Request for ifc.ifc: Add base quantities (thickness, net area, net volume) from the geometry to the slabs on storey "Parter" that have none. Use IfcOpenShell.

First a look at what the model holds.

```python
import ifcopenshell
import ifcopenshell.util.element
import ifcopenshell.util.unit

model = ifcopenshell.open("ifc.ifc")
print(model.schema)
for unit_type in ("LENGTHUNIT", "AREAUNIT", "VOLUMEUNIT"):
    print(unit_type, ifcopenshell.util.unit.calculate_unit_scale(model, unit_type))
storey = next(s for s in model.by_type("IfcBuildingStorey") if s.Name == "Parter")
slabs = [e for e in ifcopenshell.util.element.get_decomposition(storey) if e.is_a("IfcSlab")]
for e in sorted(slabs, key=lambda e: e.id()):
    print(e.id(), e.is_a(), e.Name, list(ifcopenshell.util.element.get_psets(e, qtos_only=True)), sep=" | ")
```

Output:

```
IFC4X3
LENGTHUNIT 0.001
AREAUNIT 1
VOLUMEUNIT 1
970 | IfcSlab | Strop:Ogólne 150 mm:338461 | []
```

```python
import ifcopenshell
import ifcopenshell.api.pset
import ifcopenshell.geom
import ifcopenshell.util.element
import ifcopenshell.util.shape
import ifcopenshell.util.unit

model = ifcopenshell.open("ifc.ifc")
unit_scale = ifcopenshell.util.unit.calculate_unit_scale(model)
area_scale = ifcopenshell.util.unit.calculate_unit_scale(model, "AREAUNIT")
volume_scale = ifcopenshell.util.unit.calculate_unit_scale(model, "VOLUMEUNIT")
settings = ifcopenshell.geom.settings()

storey = next(s for s in model.by_type("IfcBuildingStorey") if s.Name == "Parter")
slabs = [e for e in ifcopenshell.util.element.get_decomposition(storey) if e.is_a("IfcSlab")]

for e in sorted(slabs, key=lambda e: e.id()):
    if ifcopenshell.util.element.get_psets(e, qtos_only=True, should_inherit=False):
        continue
    # Geometry comes back in metres, in the element's own axes.
    shape = ifcopenshell.geom.create_shape(settings, e)
    values = {
        "Width": ifcopenshell.util.shape.get_z(shape.geometry) / unit_scale,
        "NetArea": ifcopenshell.util.shape.get_footprint_area(shape.geometry) / area_scale,
        "NetVolume": ifcopenshell.util.shape.get_volume(shape.geometry) / volume_scale,
    }
    qto = ifcopenshell.api.pset.add_qto(model, product=e, name="Qto_SlabBaseQuantities")
    ifcopenshell.api.pset.edit_qto(model, qto=qto, properties=values)
    print(e.id(), {k: round(v, 3) for k, v in values.items()})

model.write("ifc_rev.ifc")
```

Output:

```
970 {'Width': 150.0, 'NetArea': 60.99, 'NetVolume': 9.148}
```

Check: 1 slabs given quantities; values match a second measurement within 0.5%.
